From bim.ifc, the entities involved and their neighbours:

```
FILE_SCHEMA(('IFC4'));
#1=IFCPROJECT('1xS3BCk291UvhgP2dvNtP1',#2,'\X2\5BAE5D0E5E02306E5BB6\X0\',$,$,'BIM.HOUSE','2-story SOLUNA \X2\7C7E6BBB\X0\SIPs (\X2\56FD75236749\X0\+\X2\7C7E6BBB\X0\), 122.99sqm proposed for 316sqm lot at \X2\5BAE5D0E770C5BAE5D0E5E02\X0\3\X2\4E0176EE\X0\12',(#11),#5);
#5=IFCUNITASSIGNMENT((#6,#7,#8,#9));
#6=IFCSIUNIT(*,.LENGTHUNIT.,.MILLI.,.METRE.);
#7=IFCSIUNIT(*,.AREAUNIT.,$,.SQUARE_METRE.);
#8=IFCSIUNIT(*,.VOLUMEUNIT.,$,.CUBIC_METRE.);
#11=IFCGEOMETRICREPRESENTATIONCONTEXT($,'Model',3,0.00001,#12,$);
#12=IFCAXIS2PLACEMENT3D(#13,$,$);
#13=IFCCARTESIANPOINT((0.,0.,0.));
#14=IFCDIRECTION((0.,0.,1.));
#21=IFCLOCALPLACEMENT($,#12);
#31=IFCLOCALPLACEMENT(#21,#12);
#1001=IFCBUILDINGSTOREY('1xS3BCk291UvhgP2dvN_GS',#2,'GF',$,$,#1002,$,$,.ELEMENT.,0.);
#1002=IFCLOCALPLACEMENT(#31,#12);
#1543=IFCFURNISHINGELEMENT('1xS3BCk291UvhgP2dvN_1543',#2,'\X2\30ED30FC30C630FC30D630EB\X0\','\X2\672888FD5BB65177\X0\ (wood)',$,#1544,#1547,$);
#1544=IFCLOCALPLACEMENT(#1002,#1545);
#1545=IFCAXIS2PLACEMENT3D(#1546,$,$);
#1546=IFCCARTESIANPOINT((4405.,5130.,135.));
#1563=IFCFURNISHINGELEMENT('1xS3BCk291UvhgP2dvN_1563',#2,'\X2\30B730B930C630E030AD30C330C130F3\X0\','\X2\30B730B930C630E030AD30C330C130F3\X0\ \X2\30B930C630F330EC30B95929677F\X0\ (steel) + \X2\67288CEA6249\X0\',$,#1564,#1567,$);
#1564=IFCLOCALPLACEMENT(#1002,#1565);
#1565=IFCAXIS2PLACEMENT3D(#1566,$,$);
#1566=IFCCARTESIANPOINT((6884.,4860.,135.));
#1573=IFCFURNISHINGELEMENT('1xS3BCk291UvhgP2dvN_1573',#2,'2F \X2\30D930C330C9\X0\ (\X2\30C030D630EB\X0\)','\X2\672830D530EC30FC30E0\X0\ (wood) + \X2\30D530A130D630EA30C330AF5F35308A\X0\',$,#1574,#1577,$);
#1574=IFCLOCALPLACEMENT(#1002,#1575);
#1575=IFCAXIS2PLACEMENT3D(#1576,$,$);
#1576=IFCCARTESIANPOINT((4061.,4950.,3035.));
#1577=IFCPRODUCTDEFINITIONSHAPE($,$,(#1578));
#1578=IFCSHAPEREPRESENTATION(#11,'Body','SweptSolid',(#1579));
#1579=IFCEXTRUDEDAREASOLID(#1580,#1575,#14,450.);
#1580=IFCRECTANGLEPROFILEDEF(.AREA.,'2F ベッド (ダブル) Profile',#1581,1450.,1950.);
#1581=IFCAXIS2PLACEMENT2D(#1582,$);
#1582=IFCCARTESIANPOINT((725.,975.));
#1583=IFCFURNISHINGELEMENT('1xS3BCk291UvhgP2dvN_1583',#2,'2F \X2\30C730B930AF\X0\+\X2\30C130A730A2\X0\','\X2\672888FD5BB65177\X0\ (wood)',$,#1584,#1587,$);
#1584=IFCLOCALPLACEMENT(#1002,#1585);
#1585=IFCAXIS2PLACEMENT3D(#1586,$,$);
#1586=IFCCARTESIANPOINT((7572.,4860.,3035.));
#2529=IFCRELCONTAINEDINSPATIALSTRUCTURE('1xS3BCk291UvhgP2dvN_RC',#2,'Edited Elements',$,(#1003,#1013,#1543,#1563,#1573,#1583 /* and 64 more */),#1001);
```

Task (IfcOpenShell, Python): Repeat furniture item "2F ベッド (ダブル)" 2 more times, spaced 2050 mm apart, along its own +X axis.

```python
import ifcopenshell
import ifcopenshell.api.geometry
import ifcopenshell.api.root
import ifcopenshell.util.element
import ifcopenshell.util.placement
import ifcopenshell.util.unit

model = ifcopenshell.open("bim.ifc")
unit_scale = ifcopenshell.util.unit.calculate_unit_scale(model)


def reuse_history(source, copy):
    """copy_class also copies each property set's owner history, people and application; keep the originals."""
    for rel in copy.IsDefinedBy:
        if rel.is_a("IfcRelDefinesByProperties") and (history := rel.RelatingPropertyDefinition.OwnerHistory):
            rel.RelatingPropertyDefinition.OwnerHistory = source.OwnerHistory
            ifcopenshell.util.element.remove_deep2(model, history)


source = model.by_guid("1xS3BCk291UvhgP2dvN_1573")
base = ifcopenshell.util.placement.get_local_placement(source.ObjectPlacement)
step = base[:3, 0] * 2.05 / unit_scale

for i in range(1, 3):
    copy = ifcopenshell.api.root.copy_class(model, product=source)
    copy.Representation = ifcopenshell.util.element.copy_deep(
        model, source.Representation, exclude=["IfcGeometricRepresentationContext", "IfcRepresentationMap"]
    )
    reuse_history(source, copy)
    matrix = base.copy()
    matrix[:3, 3] += i * step
    print("added at", matrix[:3, 3].round(3) + 0.0)
    ifcopenshell.api.geometry.edit_object_placement(model, product=copy, matrix=matrix, is_si=False)

model.write("bim_updated.ifc")
```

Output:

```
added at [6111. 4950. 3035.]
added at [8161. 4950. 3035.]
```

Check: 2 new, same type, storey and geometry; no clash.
